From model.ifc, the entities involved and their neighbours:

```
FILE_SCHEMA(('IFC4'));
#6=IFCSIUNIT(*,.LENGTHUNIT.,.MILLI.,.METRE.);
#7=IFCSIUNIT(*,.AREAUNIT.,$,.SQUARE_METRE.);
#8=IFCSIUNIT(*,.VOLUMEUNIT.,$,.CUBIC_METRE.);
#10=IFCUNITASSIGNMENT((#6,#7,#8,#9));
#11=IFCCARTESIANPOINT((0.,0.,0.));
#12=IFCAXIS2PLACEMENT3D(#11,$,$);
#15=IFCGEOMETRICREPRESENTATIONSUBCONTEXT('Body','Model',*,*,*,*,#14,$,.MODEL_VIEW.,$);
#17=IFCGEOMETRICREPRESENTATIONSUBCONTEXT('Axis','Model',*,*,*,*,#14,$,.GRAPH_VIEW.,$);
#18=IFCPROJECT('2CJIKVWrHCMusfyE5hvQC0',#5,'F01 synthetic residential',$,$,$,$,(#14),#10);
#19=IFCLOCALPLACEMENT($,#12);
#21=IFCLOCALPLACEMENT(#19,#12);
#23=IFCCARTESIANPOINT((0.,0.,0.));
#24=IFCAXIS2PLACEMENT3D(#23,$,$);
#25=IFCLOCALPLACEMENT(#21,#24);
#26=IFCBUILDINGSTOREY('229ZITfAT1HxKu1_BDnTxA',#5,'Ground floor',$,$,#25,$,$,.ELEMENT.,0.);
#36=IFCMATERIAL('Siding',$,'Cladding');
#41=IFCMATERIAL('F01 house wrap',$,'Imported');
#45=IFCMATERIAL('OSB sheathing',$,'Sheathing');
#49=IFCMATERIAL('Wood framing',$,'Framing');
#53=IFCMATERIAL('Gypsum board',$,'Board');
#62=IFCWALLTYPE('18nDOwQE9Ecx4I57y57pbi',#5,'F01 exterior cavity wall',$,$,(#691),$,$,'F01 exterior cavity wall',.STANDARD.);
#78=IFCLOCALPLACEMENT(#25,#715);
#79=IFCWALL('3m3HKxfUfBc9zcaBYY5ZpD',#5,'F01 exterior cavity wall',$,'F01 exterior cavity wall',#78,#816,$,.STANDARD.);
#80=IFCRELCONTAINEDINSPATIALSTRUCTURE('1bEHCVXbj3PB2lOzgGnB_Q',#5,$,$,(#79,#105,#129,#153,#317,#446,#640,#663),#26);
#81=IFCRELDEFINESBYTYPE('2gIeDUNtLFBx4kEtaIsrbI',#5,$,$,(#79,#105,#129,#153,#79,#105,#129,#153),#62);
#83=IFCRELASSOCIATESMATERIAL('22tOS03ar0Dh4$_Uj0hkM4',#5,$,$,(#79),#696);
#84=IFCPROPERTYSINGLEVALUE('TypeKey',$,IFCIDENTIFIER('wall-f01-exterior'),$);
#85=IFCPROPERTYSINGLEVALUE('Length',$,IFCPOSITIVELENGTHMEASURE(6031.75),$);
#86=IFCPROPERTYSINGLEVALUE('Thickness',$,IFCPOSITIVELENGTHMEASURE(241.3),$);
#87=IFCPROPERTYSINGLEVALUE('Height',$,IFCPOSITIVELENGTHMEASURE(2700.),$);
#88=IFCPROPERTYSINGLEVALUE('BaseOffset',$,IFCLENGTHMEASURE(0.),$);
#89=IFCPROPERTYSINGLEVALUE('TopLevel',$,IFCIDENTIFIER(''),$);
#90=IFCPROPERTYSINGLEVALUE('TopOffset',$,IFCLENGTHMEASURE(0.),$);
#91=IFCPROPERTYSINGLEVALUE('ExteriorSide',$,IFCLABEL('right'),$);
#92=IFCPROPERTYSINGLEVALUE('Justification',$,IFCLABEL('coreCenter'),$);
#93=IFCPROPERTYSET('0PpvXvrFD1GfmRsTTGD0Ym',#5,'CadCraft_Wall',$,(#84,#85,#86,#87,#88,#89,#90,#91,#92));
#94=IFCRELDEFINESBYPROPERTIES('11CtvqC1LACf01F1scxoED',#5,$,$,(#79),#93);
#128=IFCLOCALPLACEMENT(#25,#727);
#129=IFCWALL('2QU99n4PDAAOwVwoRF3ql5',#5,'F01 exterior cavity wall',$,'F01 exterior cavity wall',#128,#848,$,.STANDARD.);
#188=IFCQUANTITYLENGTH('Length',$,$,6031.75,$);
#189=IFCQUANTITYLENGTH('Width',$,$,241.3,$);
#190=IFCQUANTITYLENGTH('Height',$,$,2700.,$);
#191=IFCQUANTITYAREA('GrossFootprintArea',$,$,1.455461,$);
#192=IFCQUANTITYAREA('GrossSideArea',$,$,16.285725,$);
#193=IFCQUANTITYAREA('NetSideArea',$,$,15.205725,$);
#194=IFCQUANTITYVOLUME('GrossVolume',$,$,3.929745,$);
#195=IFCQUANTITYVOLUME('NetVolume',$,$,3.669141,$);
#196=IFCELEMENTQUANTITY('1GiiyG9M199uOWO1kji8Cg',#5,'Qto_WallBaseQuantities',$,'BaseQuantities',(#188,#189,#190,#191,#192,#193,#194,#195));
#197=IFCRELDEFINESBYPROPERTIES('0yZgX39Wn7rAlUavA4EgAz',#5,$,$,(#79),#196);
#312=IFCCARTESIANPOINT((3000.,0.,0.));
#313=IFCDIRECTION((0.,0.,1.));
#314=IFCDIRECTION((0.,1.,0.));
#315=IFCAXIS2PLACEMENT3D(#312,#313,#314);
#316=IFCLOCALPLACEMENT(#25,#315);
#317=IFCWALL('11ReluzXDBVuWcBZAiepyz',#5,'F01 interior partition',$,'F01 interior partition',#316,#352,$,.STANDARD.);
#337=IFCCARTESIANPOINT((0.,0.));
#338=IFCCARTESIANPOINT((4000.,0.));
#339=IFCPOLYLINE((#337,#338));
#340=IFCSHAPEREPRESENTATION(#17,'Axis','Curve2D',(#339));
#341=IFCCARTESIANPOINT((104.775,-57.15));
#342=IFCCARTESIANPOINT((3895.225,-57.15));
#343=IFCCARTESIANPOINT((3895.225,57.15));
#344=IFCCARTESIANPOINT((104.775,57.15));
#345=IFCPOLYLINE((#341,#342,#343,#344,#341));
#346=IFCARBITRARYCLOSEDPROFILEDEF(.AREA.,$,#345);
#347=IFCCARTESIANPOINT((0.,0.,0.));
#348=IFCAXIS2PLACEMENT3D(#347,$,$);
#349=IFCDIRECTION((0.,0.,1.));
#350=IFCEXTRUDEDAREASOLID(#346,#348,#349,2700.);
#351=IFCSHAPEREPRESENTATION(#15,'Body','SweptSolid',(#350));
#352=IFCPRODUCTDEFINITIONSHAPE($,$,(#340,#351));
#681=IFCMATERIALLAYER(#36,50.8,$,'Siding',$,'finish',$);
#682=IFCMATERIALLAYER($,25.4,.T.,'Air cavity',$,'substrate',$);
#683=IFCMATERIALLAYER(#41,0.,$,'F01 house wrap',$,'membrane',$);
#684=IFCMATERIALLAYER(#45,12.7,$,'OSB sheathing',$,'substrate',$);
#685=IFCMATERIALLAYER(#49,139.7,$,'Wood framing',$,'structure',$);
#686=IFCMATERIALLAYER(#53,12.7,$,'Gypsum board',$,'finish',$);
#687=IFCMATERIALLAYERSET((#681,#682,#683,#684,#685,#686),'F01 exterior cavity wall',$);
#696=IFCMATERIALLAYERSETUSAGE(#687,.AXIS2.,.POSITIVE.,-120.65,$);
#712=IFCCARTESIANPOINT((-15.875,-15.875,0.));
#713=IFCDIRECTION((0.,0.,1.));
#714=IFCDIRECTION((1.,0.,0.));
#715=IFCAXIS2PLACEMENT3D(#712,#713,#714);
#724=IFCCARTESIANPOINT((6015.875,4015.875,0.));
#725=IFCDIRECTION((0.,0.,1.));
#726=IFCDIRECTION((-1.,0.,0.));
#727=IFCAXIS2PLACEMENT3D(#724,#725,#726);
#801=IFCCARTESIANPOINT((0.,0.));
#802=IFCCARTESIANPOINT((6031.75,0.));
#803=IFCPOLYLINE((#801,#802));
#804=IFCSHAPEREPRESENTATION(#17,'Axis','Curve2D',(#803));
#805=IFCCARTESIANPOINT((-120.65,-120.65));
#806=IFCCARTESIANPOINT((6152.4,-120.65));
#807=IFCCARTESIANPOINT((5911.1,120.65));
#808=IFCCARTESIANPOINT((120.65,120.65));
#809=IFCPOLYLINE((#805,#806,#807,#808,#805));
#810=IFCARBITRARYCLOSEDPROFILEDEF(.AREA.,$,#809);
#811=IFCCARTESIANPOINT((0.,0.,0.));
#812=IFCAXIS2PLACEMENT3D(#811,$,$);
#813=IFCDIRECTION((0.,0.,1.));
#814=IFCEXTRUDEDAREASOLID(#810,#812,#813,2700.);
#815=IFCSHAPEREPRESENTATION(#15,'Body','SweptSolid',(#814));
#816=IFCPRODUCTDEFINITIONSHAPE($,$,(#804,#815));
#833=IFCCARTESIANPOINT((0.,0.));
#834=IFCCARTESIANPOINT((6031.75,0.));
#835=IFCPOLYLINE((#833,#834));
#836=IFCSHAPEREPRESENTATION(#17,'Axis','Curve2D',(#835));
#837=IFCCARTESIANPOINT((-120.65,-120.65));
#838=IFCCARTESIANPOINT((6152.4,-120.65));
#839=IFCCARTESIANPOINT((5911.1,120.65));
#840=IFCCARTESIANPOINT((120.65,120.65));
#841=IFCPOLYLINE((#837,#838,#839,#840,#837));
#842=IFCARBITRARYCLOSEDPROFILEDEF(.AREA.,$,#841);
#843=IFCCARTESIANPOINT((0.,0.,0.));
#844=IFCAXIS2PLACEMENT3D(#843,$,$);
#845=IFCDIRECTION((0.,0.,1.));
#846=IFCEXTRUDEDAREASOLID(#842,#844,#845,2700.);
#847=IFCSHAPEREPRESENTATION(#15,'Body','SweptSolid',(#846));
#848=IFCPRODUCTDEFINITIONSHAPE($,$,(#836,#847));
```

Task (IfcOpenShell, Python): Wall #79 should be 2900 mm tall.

```python
import ifcopenshell
import ifcopenshell.api.pset
import ifcopenshell.geom
import ifcopenshell.util.element
import ifcopenshell.util.representation
import ifcopenshell.util.shape
import ifcopenshell.util.unit

model = ifcopenshell.open("model.ifc")
unit_scale = ifcopenshell.util.unit.calculate_unit_scale(model)
area_scale = ifcopenshell.util.unit.calculate_unit_scale(model, "AREAUNIT")
volume_scale = ifcopenshell.util.unit.calculate_unit_scale(model, "VOLUMEUNIT")
settings = ifcopenshell.geom.settings()


def volume(element):
    """Net volume in cubic metres, openings subtracted."""
    shape = ifcopenshell.geom.create_shape(settings, element)
    return ifcopenshell.util.shape.get_volume(shape.geometry)


wall = model.by_id(79)
before = volume(wall)

body = ifcopenshell.util.representation.get_representation(wall, "Model", "Body")
solid = body.Items[0]
old_height = solid.Depth
solid.Depth = 2.9 / unit_scale
after = volume(wall)
thickness = 0.2413  # wall thickness in metres

# Update the stored height, areas and volumes.
pset = model.by_id(ifcopenshell.util.element.get_pset(wall, "CadCraft_Wall", should_inherit=False)["id"])
ifcopenshell.api.pset.edit_pset(model, pset=pset, properties={
    "Height": model.create_entity("IfcPositiveLengthMeasure", solid.Depth),
})
qto = model.by_id(ifcopenshell.util.element.get_pset(wall, "Qto_WallBaseQuantities", should_inherit=False)["id"])
ifcopenshell.api.pset.edit_qto(model, qto=qto, properties={
    "Height": solid.Depth,
    "GrossSideArea": ifcopenshell.util.element.get_pset(wall, "Qto_WallBaseQuantities", "GrossSideArea") * solid.Depth / old_height,
    "NetSideArea": after / thickness / area_scale,
    "GrossVolume": ifcopenshell.util.element.get_pset(wall, "Qto_WallBaseQuantities", "GrossVolume") * solid.Depth / old_height,
    "NetVolume": after / volume_scale,
})

print(f"height {old_height:g} -> {solid.Depth:g}, volume {before:.3f} -> {after:.3f} m3")

model.write("model_updated.ifc")
```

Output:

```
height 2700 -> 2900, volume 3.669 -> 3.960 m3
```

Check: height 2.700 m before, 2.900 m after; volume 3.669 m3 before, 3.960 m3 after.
